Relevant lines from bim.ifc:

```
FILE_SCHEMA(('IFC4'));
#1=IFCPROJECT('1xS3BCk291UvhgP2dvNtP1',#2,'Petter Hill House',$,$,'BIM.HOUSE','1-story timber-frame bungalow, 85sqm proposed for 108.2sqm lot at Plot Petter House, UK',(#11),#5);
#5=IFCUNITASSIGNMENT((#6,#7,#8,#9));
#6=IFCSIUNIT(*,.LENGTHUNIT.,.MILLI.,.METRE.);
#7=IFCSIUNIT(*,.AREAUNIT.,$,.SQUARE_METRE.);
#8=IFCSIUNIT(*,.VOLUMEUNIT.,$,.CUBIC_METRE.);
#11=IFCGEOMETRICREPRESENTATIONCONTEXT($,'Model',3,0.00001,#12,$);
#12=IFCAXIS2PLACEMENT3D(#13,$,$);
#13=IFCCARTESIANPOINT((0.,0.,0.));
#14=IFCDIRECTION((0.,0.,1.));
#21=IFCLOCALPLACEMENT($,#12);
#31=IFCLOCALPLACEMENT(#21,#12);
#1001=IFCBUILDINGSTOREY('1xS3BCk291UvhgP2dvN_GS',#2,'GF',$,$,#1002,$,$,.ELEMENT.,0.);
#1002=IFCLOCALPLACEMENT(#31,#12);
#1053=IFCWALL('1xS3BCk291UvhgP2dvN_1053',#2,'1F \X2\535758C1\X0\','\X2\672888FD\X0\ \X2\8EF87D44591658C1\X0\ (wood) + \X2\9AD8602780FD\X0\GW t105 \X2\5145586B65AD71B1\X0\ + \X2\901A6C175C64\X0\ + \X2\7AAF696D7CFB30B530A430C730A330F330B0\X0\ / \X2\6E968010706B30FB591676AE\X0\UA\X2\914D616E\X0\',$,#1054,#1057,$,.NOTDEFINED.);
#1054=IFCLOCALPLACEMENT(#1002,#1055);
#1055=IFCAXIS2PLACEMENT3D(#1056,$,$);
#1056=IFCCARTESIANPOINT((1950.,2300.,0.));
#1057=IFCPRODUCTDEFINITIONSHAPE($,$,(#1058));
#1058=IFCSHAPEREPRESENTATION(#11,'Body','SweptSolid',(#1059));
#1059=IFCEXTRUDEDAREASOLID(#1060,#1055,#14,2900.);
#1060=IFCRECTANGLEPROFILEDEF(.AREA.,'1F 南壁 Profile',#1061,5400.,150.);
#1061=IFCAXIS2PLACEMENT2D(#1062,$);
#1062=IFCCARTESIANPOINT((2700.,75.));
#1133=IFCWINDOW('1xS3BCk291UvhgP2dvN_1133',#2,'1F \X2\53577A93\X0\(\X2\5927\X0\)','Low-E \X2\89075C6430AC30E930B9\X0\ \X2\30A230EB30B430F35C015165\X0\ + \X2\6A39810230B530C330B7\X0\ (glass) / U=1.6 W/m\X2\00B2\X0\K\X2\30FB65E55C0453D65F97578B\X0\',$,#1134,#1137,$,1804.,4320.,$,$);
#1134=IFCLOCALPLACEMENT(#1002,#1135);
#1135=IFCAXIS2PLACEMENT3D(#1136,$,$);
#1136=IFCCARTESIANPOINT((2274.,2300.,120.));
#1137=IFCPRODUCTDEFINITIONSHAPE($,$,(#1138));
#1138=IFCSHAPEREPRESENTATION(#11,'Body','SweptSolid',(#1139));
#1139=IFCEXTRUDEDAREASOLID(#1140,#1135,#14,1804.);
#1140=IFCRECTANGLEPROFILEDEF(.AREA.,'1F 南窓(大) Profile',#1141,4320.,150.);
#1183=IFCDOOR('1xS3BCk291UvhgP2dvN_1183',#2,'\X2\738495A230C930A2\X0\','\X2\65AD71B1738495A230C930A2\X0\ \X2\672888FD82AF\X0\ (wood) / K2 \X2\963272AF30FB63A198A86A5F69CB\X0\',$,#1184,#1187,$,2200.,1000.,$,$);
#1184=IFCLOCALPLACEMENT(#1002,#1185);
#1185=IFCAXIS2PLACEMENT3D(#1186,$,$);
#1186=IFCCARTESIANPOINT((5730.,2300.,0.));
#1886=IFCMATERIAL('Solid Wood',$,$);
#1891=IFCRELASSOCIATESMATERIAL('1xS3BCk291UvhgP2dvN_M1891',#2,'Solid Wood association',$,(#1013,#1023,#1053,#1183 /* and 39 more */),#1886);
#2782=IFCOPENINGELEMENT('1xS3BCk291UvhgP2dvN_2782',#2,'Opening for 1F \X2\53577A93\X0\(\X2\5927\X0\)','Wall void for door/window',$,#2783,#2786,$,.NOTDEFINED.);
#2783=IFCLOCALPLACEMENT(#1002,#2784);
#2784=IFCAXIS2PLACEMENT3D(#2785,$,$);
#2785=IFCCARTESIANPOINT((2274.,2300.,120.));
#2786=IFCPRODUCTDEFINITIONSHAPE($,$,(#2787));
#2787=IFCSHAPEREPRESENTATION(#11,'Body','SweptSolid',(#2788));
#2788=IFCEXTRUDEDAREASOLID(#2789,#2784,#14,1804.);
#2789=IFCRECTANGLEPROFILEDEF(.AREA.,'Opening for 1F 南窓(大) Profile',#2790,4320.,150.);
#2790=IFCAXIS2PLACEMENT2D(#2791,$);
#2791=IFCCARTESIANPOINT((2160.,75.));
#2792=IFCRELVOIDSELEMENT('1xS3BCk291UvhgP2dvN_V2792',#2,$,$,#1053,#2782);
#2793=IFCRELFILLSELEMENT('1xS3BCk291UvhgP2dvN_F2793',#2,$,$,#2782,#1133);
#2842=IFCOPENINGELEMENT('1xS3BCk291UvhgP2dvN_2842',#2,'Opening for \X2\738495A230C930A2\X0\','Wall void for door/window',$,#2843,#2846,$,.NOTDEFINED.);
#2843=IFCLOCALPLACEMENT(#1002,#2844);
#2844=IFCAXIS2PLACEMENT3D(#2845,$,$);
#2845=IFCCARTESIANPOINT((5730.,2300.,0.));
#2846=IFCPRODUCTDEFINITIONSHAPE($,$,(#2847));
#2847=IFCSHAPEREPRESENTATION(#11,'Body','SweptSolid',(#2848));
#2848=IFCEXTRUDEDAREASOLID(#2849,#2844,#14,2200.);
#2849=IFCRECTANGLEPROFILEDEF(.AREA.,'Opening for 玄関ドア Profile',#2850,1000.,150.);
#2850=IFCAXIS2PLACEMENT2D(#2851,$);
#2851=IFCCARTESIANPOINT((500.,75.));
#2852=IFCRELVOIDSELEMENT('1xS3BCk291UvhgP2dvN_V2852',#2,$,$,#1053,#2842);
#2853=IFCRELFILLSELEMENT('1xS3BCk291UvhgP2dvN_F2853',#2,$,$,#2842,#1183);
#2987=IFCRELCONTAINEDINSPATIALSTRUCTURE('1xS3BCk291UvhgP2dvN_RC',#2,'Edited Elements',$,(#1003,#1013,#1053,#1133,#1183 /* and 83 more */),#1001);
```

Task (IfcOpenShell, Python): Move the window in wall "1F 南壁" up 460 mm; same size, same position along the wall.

```python
import numpy as np
import ifcopenshell
import ifcopenshell.api.geometry
import ifcopenshell.util.placement
import ifcopenshell.util.unit

model = ifcopenshell.open("bim.ifc")
unit_scale = ifcopenshell.util.unit.calculate_unit_scale(model)

window = model.by_guid("1xS3BCk291UvhgP2dvN_1133")
opening = window.FillsVoids[0].RelatingOpeningElement
dz = 0.46 / unit_scale

shift = np.array([0.0, 0.0, dz])
# The window is not placed relative to its opening, so move both.
for product in (opening, window):
    matrix = ifcopenshell.util.placement.get_local_placement(product.ObjectPlacement)
    matrix[:3, 3] += shift
    ifcopenshell.api.geometry.edit_object_placement(model, product=product, matrix=matrix, is_si=False)

print(f"moved by {dz * unit_scale:+.3f} m")

model.write("bim_updated.ifc")
```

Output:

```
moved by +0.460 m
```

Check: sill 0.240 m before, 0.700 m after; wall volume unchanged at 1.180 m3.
